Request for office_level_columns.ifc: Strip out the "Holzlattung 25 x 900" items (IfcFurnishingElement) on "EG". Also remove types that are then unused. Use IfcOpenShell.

First a look at what the model holds.

```python
import ifcopenshell
import ifcopenshell.util.element

model = ifcopenshell.open("office_level_columns.ifc")
print(model.schema)
storey = next(s for s in model.by_type("IfcBuildingStorey") if s.Name == "EG")
furniture = [e for e in ifcopenshell.util.element.get_decomposition(storey) if e.is_a("IfcFurnishingElement")]
seen = {}
for e in furniture:
    element_type = ifcopenshell.util.element.get_type(e)
    name = element_type.Name if element_type not in (None, e) else None
    seen[name] = seen.get(name, 0) + 1
for name, count in sorted(seen.items(), key=str):
    print(count, "x", name)
```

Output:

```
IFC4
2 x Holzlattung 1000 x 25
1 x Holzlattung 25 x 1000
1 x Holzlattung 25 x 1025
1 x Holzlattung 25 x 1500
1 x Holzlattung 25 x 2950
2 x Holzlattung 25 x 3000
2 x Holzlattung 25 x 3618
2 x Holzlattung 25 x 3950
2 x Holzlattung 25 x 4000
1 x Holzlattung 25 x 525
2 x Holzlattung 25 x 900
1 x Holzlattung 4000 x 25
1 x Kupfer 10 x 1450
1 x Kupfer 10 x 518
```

```python
import ifcopenshell
import ifcopenshell.api.root
import ifcopenshell.util.element

model = ifcopenshell.open("office_level_columns.ifc")

storey = next(s for s in model.by_type("IfcBuildingStorey") if s.Name == "EG")
furniture = [e for e in ifcopenshell.util.element.get_decomposition(storey) if e.is_a("IfcFurnishingElement")]
targets = [e for e in furniture if (t := ifcopenshell.util.element.get_type(e)) not in (None, e) and t.Name == "Holzlattung 25 x 900"]
types = {ifcopenshell.util.element.get_type(e) for e in targets} - {None, *targets}

for e in targets:
    ifcopenshell.api.root.remove_product(model, product=e)
print(len(targets), "removed")

unused = [t for t in types if not ifcopenshell.util.element.get_types(t)]
for t in unused:
    ifcopenshell.api.root.remove_product(model, product=t)
print(len(unused), "unused types removed")

model.write("office_level_columns_rev.ifc")
```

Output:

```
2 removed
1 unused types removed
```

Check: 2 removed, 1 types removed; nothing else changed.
